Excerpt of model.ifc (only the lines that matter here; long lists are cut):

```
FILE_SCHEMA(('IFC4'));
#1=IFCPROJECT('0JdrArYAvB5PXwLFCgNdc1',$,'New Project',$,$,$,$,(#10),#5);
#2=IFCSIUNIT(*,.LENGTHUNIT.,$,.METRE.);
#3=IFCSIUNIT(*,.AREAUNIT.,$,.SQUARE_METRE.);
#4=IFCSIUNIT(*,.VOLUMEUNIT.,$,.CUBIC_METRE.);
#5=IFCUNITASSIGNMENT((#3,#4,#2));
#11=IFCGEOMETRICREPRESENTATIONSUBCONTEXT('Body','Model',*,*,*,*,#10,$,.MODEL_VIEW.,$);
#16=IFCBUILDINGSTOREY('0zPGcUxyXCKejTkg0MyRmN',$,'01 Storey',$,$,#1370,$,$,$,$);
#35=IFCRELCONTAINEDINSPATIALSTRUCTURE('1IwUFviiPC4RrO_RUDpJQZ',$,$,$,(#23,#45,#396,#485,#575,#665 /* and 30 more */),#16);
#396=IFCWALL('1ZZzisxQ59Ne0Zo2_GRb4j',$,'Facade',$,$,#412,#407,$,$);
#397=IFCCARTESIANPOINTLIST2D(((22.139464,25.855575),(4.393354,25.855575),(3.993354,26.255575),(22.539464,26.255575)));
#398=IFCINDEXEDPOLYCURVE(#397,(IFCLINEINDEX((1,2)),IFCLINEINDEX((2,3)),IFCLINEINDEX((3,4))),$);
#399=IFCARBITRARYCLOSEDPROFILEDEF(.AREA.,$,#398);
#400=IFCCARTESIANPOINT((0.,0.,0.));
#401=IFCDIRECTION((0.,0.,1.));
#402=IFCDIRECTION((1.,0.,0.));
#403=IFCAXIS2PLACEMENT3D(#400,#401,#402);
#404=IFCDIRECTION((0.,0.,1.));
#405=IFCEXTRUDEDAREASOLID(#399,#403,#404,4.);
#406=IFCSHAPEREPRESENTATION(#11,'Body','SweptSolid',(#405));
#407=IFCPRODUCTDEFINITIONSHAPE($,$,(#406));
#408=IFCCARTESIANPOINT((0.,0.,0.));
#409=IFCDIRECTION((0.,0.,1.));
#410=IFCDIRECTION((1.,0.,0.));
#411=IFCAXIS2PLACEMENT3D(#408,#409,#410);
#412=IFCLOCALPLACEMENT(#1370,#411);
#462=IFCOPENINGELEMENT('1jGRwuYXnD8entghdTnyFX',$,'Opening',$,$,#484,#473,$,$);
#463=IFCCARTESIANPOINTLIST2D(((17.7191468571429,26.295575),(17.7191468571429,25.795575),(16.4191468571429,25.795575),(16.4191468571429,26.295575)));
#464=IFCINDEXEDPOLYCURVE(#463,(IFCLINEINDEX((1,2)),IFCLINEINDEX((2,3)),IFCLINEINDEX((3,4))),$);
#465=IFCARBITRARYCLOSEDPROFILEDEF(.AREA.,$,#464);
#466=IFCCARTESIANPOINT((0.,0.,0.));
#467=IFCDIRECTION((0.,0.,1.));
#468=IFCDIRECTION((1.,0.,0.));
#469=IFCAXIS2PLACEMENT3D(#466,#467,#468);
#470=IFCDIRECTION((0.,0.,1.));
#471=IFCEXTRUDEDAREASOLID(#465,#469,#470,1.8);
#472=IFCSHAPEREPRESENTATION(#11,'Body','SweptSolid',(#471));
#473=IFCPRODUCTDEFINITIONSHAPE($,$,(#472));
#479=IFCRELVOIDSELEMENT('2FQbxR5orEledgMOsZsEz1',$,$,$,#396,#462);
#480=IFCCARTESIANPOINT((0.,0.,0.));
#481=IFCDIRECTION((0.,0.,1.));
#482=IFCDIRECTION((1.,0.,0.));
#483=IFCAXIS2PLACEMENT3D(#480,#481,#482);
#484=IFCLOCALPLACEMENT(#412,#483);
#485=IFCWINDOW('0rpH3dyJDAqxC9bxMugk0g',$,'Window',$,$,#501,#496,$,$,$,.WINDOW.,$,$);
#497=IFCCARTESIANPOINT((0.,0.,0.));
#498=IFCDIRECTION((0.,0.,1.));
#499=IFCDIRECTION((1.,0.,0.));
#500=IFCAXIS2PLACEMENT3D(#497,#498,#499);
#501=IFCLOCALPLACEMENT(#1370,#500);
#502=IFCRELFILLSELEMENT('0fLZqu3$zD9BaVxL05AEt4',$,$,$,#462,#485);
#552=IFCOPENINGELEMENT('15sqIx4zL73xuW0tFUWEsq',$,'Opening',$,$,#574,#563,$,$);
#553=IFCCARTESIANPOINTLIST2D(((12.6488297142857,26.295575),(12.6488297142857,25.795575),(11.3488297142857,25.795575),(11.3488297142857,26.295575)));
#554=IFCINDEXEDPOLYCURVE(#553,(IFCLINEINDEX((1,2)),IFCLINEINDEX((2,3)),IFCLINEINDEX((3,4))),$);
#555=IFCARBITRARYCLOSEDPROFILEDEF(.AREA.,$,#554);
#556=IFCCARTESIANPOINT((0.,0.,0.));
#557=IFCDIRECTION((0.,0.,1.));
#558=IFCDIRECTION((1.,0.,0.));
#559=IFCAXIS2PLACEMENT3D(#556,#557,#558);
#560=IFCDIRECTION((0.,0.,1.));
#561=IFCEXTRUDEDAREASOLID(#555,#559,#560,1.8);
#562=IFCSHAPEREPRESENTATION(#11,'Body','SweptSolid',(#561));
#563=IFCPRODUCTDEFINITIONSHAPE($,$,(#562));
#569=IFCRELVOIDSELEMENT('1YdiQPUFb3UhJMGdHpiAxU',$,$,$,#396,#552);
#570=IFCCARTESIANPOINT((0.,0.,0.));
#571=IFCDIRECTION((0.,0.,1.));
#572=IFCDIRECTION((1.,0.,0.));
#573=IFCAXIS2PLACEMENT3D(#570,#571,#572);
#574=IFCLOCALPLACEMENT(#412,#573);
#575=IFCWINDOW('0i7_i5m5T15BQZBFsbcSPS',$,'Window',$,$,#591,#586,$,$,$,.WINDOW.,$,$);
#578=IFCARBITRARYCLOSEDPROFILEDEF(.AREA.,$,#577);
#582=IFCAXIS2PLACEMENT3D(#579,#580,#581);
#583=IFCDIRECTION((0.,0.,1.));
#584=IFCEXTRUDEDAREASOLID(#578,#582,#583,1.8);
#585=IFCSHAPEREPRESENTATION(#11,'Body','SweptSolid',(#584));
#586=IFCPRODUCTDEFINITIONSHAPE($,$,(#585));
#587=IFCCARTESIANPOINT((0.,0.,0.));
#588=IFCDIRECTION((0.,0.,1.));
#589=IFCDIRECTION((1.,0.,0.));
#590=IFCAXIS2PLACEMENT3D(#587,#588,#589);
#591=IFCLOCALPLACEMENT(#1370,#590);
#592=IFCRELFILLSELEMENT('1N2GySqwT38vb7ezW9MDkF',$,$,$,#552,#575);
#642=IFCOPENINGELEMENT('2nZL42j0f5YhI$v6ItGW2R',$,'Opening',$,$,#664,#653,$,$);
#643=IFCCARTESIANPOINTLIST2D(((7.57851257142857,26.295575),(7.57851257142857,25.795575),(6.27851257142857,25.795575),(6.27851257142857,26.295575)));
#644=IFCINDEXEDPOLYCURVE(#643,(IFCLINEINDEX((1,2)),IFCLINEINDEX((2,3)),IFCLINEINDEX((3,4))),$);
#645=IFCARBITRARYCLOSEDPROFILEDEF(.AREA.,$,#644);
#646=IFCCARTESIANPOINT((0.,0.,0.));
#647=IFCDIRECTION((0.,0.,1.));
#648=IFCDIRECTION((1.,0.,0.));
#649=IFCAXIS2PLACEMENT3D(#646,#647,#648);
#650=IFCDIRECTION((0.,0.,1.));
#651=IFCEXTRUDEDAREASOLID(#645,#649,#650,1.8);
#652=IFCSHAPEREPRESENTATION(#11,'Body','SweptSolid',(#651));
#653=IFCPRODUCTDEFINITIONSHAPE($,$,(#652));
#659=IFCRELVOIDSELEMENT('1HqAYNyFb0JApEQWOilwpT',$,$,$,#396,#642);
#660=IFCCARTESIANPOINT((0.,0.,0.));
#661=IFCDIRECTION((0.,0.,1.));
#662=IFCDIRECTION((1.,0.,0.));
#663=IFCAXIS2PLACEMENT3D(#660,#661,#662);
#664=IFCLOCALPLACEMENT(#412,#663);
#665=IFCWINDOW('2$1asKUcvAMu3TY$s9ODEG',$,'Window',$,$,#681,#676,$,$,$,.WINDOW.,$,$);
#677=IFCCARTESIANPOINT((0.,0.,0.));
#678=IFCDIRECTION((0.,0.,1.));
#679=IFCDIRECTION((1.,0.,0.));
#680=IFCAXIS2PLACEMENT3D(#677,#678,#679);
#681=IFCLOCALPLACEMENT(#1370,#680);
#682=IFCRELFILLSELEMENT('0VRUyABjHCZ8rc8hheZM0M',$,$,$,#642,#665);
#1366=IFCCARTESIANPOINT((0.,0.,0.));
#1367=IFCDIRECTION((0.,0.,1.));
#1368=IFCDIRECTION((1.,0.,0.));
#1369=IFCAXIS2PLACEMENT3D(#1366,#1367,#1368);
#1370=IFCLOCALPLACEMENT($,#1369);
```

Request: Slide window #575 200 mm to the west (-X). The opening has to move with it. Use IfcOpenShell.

```python
import ifcopenshell
import ifcopenshell.api.geometry
import ifcopenshell.util.placement
import ifcopenshell.util.unit

model = ifcopenshell.open("model.ifc")
unit_scale = ifcopenshell.util.unit.calculate_unit_scale(model)

window = model.by_guid("0i7_i5m5T15BQZBFsbcSPS")
opening = window.FillsVoids[0].RelatingOpeningElement
wall = opening.VoidsElements[0].RelatingBuildingElement

wall_matrix = ifcopenshell.util.placement.get_local_placement(wall.ObjectPlacement)
shift = wall_matrix[:3, 0] * -0.2 / unit_scale
before = ifcopenshell.util.placement.get_local_placement(window.ObjectPlacement)[:3, 3].copy()

# The window is not placed relative to its opening, so move both.
for product in (opening, window):
    matrix = ifcopenshell.util.placement.get_local_placement(product.ObjectPlacement)
    matrix[:3, 3] += shift
    ifcopenshell.api.geometry.edit_object_placement(model, product=product, matrix=matrix, is_si=False)

after = ifcopenshell.util.placement.get_local_placement(window.ObjectPlacement)[:3, 3]
print("window moved by", (after - before).round(3) + 0.0)

model.write("model_v2.ifc")
```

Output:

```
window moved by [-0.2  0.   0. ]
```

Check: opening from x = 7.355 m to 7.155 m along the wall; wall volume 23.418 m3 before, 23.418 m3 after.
